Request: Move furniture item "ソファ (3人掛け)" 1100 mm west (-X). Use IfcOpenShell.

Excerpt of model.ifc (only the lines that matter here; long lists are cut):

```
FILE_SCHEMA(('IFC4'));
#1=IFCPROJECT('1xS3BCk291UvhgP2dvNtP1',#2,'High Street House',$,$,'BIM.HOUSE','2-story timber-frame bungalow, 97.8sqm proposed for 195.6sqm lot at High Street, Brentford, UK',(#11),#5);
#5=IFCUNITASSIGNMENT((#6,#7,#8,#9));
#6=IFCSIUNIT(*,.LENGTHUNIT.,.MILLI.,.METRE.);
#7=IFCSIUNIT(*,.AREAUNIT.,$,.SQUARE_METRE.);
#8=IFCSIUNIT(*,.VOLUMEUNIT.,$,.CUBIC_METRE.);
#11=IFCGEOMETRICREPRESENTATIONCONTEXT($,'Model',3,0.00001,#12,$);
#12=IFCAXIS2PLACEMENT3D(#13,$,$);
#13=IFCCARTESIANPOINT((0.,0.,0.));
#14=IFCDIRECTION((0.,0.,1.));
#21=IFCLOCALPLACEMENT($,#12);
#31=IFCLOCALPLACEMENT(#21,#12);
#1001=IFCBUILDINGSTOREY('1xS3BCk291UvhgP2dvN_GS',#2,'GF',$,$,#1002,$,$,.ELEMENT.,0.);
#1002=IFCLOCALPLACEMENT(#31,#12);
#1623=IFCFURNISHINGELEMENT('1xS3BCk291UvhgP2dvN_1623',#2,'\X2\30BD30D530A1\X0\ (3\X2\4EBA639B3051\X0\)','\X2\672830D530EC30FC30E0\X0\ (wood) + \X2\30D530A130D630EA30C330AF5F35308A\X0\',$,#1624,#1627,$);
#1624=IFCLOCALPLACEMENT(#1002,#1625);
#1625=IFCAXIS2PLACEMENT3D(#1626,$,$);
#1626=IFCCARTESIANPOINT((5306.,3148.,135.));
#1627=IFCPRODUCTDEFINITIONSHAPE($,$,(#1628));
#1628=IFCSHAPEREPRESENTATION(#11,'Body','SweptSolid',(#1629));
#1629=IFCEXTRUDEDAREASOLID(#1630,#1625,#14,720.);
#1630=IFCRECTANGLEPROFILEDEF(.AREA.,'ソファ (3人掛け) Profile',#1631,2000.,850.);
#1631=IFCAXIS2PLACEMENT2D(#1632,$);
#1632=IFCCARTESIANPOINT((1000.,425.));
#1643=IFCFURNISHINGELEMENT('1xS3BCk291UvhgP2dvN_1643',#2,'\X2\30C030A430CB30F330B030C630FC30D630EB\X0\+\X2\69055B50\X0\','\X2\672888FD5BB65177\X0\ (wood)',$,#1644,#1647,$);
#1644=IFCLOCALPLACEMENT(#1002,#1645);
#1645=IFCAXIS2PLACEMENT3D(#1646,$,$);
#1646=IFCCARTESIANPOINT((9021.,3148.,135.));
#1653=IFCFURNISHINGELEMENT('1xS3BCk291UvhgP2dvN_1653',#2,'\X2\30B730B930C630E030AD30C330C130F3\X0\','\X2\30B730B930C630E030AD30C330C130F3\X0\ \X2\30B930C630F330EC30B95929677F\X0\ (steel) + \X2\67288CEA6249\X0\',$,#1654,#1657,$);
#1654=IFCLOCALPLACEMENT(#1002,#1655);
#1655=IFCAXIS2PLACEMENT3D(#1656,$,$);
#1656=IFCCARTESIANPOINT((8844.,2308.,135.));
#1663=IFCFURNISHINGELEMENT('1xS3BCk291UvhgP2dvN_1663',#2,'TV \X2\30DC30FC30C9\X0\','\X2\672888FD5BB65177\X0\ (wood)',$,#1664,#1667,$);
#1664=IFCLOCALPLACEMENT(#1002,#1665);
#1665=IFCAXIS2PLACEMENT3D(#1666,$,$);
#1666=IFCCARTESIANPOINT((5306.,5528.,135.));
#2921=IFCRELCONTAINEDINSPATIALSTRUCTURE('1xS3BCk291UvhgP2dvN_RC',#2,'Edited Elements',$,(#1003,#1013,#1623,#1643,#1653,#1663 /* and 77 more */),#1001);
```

```python
import ifcopenshell
import ifcopenshell.api.geometry
import ifcopenshell.util.placement
import ifcopenshell.util.unit

model = ifcopenshell.open("model.ifc")
unit_scale = ifcopenshell.util.unit.calculate_unit_scale(model)

item = model.by_id(1623)
matrix = ifcopenshell.util.placement.get_local_placement(item.ObjectPlacement)
matrix[0, 3] -= 1.1 / unit_scale
ifcopenshell.api.geometry.edit_object_placement(model, product=item, matrix=matrix, is_si=False)

print(ifcopenshell.util.placement.get_local_placement(item.ObjectPlacement).round(3) + 0.0)

model.write("model_v2.ifc")
```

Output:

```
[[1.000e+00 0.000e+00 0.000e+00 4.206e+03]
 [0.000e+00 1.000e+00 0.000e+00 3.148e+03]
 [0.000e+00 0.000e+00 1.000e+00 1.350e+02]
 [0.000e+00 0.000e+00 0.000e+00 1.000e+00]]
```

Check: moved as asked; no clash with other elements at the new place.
